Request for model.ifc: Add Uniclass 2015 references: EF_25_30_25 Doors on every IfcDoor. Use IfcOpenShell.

First a look at what the model holds.

```python
import ifcopenshell

model = ifcopenshell.open("model.ifc")
print(model.schema)
print("classifications:", [c.Name for c in model.by_type("IfcClassification")])
for ifc_class in ("IfcDoor", "IfcRoof", "IfcStair", "IfcWall", "IfcWindow"):
    print(ifc_class, len(model.by_type(ifc_class)))
```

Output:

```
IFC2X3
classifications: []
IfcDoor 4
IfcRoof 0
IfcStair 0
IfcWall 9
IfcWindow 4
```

```python
import ifcopenshell
import ifcopenshell.api.classification

model = ifcopenshell.open("model.ifc")

# IFC2X3 requires Source and Edition and has no link from the project to the system.
system = model.create_entity("IfcClassification", Source="NBS", Edition="2015", Name="Uniclass 2015")

codes = {
    "IfcDoor": ("EF_25_30_25", "Doors"),
}
for ifc_class, (code, name) in codes.items():
    products = model.by_type(ifc_class)
    ifcopenshell.api.classification.add_reference(
        model, products=products, classification=system, identification=code, name=name
    )
    print(code, len(products))

model.write("model-out.ifc")
```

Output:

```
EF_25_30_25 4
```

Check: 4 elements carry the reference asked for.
